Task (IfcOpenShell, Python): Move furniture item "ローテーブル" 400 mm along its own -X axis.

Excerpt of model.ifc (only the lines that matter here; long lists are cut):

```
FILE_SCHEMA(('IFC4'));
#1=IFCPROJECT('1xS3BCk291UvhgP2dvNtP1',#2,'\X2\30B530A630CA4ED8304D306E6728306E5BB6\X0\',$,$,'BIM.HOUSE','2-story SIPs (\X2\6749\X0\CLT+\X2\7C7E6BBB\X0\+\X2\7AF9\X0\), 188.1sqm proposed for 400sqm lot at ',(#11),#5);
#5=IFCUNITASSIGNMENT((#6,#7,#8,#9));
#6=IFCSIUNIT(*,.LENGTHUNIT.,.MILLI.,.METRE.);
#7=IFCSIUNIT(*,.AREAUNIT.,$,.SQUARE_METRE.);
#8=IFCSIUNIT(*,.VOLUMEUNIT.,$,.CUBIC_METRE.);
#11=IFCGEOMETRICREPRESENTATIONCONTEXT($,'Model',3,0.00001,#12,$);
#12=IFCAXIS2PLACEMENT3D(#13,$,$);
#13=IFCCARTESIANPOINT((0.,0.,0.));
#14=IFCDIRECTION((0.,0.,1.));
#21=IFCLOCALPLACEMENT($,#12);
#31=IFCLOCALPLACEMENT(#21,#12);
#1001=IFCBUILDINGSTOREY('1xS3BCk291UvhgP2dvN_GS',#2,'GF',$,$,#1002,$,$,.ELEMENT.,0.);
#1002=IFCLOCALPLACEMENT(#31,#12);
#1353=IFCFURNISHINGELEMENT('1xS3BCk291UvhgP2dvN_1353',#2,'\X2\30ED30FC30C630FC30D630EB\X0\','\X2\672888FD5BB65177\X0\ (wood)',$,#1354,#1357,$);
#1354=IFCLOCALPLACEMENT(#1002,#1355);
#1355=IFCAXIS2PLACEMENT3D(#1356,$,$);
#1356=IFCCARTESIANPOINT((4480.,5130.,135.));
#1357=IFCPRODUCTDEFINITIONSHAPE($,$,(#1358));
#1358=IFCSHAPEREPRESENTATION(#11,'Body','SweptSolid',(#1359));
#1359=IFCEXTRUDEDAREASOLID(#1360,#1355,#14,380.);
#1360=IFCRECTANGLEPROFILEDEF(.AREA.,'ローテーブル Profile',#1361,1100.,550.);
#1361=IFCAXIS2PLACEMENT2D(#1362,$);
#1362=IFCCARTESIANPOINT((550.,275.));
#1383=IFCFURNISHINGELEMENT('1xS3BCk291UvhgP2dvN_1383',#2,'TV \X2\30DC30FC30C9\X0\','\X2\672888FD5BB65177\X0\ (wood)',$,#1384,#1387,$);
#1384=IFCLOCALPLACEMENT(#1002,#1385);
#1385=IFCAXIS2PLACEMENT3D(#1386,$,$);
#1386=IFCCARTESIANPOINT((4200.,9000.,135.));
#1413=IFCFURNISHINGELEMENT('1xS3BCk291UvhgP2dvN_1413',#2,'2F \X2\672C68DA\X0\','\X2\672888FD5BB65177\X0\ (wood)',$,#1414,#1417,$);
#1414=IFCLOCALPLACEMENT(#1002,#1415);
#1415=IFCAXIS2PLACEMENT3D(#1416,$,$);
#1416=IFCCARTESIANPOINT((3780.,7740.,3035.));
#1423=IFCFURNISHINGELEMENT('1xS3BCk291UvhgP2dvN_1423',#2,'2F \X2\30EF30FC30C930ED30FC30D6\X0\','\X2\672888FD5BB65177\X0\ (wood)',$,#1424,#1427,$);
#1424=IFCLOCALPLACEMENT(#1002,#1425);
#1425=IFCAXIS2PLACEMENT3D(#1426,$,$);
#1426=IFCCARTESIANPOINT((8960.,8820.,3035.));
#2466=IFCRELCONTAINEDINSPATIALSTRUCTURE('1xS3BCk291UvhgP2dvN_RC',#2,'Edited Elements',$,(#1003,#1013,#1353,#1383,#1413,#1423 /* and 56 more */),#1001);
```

```python
import ifcopenshell
import ifcopenshell.api.geometry
import ifcopenshell.util.placement
import ifcopenshell.util.unit

model = ifcopenshell.open("model.ifc")
unit_scale = ifcopenshell.util.unit.calculate_unit_scale(model)

item = model.by_guid("1xS3BCk291UvhgP2dvN_1353")
matrix = ifcopenshell.util.placement.get_local_placement(item.ObjectPlacement)
matrix[:3, 3] -= matrix[:3, 0] * 0.4 / unit_scale
ifcopenshell.api.geometry.edit_object_placement(model, product=item, matrix=matrix, is_si=False)

print(ifcopenshell.util.placement.get_local_placement(item.ObjectPlacement).round(3) + 0.0)

model.write("model_v2.ifc")
```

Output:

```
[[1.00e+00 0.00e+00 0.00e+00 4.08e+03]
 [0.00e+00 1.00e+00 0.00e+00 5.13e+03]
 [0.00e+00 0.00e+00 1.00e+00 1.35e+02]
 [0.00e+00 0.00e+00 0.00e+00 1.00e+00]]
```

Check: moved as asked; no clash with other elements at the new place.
